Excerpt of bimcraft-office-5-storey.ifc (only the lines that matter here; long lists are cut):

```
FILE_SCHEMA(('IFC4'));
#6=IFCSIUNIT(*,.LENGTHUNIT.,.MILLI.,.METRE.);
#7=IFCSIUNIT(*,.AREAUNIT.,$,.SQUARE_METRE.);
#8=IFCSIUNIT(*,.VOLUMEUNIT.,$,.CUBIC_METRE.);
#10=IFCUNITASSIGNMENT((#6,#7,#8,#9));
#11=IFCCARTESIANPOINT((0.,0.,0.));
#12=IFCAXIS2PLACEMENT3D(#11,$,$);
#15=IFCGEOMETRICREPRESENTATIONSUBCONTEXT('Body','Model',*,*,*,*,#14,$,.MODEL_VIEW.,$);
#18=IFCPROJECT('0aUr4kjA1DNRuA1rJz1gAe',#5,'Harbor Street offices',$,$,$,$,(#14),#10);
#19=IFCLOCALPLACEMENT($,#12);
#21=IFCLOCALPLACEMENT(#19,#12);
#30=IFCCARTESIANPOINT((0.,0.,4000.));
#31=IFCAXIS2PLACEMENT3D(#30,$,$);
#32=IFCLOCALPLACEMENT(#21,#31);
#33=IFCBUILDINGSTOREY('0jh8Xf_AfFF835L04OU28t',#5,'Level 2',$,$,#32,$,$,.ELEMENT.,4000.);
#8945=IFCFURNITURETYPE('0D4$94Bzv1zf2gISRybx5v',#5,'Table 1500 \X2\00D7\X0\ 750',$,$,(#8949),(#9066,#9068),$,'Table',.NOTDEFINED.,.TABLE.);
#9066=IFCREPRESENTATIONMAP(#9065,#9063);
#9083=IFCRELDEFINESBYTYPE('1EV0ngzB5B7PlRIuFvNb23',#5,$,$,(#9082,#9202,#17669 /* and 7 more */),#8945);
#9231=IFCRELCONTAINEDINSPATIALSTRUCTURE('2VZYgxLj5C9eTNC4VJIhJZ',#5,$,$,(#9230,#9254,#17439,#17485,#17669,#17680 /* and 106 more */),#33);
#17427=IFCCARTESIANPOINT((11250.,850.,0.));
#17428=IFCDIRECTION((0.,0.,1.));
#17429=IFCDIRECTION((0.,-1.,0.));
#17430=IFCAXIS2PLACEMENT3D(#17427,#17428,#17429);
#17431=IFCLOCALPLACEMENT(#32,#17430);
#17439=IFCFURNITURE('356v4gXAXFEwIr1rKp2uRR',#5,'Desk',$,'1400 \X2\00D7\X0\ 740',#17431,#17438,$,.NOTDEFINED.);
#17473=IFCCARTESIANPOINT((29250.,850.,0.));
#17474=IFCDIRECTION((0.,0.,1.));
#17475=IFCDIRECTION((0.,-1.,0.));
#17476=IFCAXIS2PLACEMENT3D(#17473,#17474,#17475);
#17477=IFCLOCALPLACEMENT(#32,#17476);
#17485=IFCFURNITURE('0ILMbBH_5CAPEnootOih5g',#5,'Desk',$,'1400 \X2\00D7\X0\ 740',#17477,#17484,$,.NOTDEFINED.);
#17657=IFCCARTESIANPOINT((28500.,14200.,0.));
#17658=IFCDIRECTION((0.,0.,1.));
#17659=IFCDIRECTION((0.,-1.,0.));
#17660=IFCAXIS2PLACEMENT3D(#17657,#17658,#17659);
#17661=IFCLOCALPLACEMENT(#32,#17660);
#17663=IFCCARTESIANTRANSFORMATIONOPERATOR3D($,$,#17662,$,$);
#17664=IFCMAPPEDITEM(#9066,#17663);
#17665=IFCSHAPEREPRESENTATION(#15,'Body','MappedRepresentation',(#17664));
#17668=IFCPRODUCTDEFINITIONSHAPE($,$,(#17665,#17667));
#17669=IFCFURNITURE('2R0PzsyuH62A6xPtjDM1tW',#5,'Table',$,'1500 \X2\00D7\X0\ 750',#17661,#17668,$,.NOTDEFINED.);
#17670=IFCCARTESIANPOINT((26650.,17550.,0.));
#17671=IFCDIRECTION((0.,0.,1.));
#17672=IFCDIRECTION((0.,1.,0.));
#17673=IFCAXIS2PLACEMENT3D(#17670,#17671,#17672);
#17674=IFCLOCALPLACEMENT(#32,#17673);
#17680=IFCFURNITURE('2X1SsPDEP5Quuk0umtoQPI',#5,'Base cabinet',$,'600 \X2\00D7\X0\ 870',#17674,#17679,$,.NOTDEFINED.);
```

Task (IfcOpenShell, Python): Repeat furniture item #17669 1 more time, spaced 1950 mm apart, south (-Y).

```python
import numpy as np
import ifcopenshell
import ifcopenshell.api.geometry
import ifcopenshell.api.root
import ifcopenshell.util.element
import ifcopenshell.util.placement
import ifcopenshell.util.unit

model = ifcopenshell.open("bimcraft-office-5-storey.ifc")
unit_scale = ifcopenshell.util.unit.calculate_unit_scale(model)

source = model.by_id(17669)
base = ifcopenshell.util.placement.get_local_placement(source.ObjectPlacement)
step = np.array([0.0, -1.0, 0.0]) * 1.95 / unit_scale

for i in range(1, 2):
    copy = ifcopenshell.api.root.copy_class(model, product=source)
    copy.Representation = ifcopenshell.util.element.copy_deep(
        model, source.Representation, exclude=["IfcGeometricRepresentationContext", "IfcRepresentationMap"]
    )
    matrix = base.copy()
    matrix[:3, 3] += i * step
    print("added at", matrix[:3, 3].round(3) + 0.0)
    ifcopenshell.api.geometry.edit_object_placement(model, product=copy, matrix=matrix, is_si=False)

model.write("bimcraft-office-5-storey_edited.ifc")
```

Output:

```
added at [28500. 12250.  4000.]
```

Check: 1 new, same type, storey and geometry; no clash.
